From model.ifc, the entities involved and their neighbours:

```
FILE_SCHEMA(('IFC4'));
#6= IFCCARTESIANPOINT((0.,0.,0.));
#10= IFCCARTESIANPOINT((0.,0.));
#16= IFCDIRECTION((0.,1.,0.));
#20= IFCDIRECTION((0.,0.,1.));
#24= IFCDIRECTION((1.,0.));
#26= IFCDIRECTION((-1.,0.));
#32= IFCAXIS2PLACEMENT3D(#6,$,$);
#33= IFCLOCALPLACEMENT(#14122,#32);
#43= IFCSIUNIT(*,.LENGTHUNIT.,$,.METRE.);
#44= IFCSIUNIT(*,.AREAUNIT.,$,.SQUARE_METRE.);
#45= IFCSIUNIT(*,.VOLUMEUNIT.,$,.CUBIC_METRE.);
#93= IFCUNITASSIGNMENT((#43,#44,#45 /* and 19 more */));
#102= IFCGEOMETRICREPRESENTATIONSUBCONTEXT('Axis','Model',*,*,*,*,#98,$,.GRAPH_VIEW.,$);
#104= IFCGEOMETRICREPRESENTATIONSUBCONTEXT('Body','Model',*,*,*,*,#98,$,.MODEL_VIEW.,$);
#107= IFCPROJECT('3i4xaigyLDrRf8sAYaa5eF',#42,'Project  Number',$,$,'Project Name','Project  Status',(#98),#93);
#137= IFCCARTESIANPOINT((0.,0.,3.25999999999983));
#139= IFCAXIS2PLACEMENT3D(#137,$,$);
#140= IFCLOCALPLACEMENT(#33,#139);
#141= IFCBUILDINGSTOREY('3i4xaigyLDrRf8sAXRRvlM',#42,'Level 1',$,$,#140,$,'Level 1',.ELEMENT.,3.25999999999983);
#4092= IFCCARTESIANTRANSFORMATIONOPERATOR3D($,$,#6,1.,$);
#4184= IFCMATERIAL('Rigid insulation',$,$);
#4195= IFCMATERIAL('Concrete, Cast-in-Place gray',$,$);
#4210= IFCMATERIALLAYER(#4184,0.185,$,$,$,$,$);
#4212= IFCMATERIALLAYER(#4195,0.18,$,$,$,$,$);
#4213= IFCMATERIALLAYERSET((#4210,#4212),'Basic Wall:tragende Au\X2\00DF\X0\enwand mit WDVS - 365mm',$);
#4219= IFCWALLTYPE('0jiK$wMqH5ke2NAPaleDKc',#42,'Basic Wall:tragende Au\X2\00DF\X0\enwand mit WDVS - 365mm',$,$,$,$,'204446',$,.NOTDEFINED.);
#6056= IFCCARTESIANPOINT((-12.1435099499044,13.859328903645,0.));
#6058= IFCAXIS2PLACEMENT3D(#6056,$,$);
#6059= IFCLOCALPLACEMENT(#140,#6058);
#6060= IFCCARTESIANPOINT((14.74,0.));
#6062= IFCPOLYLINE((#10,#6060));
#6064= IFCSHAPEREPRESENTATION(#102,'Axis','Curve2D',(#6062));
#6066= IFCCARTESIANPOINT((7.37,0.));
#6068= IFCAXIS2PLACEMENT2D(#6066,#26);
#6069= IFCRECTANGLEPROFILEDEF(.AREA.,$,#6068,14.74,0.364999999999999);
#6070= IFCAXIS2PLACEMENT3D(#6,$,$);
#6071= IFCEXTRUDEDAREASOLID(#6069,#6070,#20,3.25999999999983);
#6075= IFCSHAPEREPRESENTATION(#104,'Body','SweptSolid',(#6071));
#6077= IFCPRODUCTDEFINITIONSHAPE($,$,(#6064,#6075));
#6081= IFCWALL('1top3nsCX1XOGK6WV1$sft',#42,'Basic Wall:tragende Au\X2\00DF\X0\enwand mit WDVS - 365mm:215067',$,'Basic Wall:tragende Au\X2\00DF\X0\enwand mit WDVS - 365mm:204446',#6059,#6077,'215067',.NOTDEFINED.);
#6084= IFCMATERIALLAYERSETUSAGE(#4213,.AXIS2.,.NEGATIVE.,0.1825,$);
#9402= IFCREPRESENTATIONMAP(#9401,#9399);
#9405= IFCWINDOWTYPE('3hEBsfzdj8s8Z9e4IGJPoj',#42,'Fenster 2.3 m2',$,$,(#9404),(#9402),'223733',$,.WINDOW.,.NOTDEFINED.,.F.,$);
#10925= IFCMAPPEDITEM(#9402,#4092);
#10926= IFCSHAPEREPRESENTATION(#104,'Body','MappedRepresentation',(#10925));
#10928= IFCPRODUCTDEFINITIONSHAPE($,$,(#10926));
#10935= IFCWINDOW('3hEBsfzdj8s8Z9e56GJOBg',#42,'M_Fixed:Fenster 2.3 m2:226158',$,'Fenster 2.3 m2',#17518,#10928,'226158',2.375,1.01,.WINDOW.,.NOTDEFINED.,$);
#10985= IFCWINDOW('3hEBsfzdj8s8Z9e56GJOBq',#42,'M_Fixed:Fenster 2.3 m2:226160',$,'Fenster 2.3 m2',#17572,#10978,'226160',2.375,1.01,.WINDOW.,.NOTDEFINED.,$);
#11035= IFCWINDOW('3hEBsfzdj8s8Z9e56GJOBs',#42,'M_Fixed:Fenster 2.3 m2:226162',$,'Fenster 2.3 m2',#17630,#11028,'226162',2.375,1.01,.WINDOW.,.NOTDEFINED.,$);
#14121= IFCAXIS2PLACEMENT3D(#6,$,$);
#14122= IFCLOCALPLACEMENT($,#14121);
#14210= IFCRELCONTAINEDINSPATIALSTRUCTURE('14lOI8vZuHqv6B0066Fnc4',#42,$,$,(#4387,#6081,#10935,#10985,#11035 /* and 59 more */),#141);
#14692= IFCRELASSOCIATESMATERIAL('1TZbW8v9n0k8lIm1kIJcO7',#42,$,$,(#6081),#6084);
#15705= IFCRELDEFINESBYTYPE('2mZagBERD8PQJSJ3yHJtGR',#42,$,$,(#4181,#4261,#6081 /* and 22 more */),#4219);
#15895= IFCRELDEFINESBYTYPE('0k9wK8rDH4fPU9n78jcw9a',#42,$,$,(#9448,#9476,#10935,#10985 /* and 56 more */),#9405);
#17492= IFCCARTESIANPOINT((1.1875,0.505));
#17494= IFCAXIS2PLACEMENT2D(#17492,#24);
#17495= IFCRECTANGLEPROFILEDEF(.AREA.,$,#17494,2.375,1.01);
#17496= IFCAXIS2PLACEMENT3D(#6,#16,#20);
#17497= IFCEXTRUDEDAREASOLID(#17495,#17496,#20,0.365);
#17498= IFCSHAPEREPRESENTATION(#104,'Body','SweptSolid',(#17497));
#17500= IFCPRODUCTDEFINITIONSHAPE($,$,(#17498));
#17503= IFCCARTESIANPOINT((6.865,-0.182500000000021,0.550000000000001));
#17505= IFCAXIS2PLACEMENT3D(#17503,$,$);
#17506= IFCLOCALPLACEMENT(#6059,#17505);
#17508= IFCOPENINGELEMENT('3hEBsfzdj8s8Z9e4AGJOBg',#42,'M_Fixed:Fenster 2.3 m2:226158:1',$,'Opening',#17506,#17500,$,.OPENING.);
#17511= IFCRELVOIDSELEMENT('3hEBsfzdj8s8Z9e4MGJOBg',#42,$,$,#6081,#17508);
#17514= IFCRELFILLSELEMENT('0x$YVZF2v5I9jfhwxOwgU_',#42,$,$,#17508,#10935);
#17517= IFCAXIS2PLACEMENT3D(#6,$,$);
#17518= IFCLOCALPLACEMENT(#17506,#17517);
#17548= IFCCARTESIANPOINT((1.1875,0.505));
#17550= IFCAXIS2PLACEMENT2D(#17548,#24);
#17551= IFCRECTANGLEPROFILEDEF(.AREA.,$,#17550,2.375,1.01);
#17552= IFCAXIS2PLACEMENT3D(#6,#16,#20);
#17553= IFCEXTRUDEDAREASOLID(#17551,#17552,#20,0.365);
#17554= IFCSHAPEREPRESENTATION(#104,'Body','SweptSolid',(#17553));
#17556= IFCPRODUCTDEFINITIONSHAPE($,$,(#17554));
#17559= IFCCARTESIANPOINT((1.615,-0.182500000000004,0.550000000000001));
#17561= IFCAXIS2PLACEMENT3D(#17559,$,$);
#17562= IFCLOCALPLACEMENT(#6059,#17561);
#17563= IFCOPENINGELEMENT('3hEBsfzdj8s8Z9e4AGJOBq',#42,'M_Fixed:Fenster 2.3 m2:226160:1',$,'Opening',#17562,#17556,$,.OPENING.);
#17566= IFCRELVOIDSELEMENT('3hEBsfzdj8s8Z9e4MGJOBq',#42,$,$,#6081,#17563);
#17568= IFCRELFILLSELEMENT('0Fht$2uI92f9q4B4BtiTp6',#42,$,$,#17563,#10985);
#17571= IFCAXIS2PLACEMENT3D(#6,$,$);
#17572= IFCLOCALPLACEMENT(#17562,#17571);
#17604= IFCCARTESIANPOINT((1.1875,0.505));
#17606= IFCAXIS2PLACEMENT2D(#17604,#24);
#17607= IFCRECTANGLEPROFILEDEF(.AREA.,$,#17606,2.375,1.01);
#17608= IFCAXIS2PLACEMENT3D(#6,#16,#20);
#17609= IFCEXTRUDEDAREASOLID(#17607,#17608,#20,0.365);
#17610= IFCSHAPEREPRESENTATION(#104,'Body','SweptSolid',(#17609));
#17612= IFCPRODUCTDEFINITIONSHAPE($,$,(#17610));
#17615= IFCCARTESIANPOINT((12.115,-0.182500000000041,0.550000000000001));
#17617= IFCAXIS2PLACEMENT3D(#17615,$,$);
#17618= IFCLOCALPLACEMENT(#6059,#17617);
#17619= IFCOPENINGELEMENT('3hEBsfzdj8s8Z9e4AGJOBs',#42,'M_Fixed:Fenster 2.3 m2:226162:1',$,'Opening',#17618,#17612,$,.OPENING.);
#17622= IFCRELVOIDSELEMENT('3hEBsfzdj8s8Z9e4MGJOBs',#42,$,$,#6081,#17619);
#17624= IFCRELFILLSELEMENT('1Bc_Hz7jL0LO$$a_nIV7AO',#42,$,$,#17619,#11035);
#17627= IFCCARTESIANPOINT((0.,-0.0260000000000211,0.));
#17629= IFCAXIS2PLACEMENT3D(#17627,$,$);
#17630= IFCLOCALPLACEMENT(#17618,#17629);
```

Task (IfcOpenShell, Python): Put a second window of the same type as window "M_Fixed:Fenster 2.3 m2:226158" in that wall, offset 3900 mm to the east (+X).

```python
import ifcopenshell
import ifcopenshell.api.feature
import ifcopenshell.api.geometry
import ifcopenshell.api.root
import ifcopenshell.geom
import ifcopenshell.util.element
import ifcopenshell.util.placement
import ifcopenshell.util.shape
import ifcopenshell.util.unit

model = ifcopenshell.open("model.ifc")
unit_scale = ifcopenshell.util.unit.calculate_unit_scale(model)
settings = ifcopenshell.geom.settings()


def volume(element):
    """Net volume in cubic metres, openings subtracted."""
    shape = ifcopenshell.geom.create_shape(settings, element)
    return ifcopenshell.util.shape.get_volume(shape.geometry)


def reuse_history(source, copy):
    """copy_class also copies each property set's owner history, people and application; keep the originals."""
    for rel in copy.IsDefinedBy:
        if rel.is_a("IfcRelDefinesByProperties") and (history := rel.RelatingPropertyDefinition.OwnerHistory):
            rel.RelatingPropertyDefinition.OwnerHistory = source.OwnerHistory
            ifcopenshell.util.element.remove_deep2(model, history)


window = model.by_guid("3hEBsfzdj8s8Z9e56GJOBg")
opening = window.FillsVoids[0].RelatingOpeningElement
wall = opening.VoidsElements[0].RelatingBuildingElement
before = volume(wall)
shift = ifcopenshell.util.placement.get_local_placement(wall.ObjectPlacement)[:3, 0] * 3.9 / unit_scale

# copy_class copies the void relationship, type, container and properties, but no geometry.
new_opening = ifcopenshell.api.root.copy_class(model, product=opening)
new_opening.Representation = ifcopenshell.util.element.copy_deep(
    model, opening.Representation, exclude=["IfcGeometricRepresentationContext", "IfcRepresentationMap"]
)
new_opening.Name = "M_Fixed:Fenster 2.3 m2"
new_window = ifcopenshell.api.root.copy_class(model, product=window)
new_window.Representation = ifcopenshell.util.element.copy_deep(
    model, window.Representation, exclude=["IfcGeometricRepresentationContext", "IfcRepresentationMap"]
)
new_window.Name = "M_Fixed:Fenster 2.3 m2"
new_window.Tag = None
reuse_history(window, new_window)
ifcopenshell.api.feature.add_filling(model, opening=new_opening, element=new_window)

for old, new in ((opening, new_opening), (window, new_window)):
    matrix = ifcopenshell.util.placement.get_local_placement(old.ObjectPlacement)
    matrix[:3, 3] += shift
    ifcopenshell.api.geometry.edit_object_placement(model, product=new, matrix=matrix, is_si=False)

after = volume(wall)

print(f"wall volume {before:.3f} -> {after:.3f} m3")

model.write("model_edited.ifc")
```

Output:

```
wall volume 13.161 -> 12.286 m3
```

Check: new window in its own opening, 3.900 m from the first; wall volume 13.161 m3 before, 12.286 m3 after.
